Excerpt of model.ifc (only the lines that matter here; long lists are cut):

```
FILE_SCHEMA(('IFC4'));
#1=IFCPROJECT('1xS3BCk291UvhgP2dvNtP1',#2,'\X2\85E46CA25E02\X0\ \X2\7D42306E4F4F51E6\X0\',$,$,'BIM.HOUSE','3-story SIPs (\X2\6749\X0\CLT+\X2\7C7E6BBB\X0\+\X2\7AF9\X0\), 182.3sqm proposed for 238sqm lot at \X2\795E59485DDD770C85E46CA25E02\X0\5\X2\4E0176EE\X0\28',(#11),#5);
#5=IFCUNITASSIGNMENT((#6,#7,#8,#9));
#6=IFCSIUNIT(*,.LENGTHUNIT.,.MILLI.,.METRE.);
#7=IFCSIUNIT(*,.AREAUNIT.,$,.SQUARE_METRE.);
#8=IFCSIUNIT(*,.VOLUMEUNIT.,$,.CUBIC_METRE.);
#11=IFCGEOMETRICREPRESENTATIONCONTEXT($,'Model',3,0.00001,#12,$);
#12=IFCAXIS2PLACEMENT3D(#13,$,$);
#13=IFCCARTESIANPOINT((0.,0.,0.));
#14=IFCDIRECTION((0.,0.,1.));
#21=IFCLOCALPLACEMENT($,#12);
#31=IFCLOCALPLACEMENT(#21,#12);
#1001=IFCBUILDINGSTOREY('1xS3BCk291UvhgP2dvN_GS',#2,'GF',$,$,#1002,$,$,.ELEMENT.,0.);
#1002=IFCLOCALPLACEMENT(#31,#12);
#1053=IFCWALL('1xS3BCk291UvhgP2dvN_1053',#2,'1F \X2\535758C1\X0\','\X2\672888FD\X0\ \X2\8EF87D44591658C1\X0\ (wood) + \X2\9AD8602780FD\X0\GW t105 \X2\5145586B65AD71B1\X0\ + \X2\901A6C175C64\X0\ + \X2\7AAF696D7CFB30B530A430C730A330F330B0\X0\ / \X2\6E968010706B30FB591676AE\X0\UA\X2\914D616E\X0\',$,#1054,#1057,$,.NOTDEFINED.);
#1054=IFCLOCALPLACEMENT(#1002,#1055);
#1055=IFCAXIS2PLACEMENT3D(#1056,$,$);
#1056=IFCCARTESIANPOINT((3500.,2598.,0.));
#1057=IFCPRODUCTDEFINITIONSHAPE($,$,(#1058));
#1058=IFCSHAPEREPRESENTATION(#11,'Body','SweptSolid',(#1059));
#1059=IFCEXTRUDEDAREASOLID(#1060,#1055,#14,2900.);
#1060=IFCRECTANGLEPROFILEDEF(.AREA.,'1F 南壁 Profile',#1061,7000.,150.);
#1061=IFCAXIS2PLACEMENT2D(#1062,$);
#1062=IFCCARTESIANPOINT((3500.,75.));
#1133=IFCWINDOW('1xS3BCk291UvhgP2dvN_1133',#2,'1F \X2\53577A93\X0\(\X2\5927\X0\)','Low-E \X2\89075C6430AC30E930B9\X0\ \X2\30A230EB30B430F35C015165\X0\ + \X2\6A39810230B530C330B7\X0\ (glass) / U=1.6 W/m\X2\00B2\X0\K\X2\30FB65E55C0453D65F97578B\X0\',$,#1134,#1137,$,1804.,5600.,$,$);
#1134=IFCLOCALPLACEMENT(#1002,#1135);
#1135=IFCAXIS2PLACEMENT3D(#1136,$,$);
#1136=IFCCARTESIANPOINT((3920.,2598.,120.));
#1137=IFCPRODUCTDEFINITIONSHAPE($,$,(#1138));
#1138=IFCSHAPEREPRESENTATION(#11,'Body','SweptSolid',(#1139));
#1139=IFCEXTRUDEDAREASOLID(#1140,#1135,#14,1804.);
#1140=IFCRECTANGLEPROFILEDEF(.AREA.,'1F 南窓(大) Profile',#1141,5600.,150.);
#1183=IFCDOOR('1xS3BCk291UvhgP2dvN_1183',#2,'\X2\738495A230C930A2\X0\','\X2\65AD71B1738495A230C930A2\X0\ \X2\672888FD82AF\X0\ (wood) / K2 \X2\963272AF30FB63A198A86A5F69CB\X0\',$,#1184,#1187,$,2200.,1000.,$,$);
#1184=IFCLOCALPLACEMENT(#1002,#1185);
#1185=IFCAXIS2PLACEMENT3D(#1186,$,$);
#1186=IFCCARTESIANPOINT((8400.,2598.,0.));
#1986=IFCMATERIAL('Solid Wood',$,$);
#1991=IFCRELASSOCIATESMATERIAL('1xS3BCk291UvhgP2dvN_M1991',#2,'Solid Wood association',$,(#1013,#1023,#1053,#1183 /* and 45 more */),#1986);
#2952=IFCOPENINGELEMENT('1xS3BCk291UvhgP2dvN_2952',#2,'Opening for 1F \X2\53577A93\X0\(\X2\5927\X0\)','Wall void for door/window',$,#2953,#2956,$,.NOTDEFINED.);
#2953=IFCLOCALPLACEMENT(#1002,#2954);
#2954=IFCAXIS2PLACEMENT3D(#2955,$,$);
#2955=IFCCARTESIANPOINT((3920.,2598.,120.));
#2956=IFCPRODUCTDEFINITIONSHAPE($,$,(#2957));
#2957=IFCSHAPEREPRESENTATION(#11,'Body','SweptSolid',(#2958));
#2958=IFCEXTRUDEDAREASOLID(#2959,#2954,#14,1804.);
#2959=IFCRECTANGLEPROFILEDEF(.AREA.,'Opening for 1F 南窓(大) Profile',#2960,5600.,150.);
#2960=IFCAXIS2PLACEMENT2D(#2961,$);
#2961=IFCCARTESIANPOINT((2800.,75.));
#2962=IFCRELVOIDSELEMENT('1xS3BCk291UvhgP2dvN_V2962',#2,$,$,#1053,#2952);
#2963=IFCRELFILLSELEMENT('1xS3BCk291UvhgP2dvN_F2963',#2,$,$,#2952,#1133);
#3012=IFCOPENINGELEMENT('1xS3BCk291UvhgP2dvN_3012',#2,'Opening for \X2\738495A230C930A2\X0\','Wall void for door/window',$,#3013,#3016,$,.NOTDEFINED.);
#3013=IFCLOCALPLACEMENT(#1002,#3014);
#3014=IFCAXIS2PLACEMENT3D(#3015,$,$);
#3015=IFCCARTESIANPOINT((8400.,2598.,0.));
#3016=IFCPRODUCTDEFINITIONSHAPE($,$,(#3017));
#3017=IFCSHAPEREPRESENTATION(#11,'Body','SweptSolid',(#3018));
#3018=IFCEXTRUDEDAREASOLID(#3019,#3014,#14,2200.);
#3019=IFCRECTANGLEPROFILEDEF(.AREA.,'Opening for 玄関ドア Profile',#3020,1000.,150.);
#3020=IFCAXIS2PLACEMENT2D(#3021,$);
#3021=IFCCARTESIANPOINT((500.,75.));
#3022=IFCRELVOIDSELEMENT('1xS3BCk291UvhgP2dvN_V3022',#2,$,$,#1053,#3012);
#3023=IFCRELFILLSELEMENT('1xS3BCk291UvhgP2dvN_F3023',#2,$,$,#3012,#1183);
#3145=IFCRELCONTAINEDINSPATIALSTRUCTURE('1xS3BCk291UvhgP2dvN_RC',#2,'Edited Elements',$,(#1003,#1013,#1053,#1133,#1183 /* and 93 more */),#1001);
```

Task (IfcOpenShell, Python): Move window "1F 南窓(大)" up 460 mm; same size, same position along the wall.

```python
import numpy as np
import ifcopenshell
import ifcopenshell.api.geometry
import ifcopenshell.util.placement
import ifcopenshell.util.unit

model = ifcopenshell.open("model.ifc")
unit_scale = ifcopenshell.util.unit.calculate_unit_scale(model)

window = model.by_guid("1xS3BCk291UvhgP2dvN_1133")
opening = window.FillsVoids[0].RelatingOpeningElement
dz = 0.46 / unit_scale

shift = np.array([0.0, 0.0, dz])
# The window is not placed relative to its opening, so move both.
for product in (opening, window):
    matrix = ifcopenshell.util.placement.get_local_placement(product.ObjectPlacement)
    matrix[:3, 3] += shift
    ifcopenshell.api.geometry.edit_object_placement(model, product=product, matrix=matrix, is_si=False)

print(f"moved by {dz * unit_scale:+.3f} m")

model.write("model_v2.ifc")
```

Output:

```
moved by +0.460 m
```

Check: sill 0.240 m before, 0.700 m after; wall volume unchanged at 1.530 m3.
